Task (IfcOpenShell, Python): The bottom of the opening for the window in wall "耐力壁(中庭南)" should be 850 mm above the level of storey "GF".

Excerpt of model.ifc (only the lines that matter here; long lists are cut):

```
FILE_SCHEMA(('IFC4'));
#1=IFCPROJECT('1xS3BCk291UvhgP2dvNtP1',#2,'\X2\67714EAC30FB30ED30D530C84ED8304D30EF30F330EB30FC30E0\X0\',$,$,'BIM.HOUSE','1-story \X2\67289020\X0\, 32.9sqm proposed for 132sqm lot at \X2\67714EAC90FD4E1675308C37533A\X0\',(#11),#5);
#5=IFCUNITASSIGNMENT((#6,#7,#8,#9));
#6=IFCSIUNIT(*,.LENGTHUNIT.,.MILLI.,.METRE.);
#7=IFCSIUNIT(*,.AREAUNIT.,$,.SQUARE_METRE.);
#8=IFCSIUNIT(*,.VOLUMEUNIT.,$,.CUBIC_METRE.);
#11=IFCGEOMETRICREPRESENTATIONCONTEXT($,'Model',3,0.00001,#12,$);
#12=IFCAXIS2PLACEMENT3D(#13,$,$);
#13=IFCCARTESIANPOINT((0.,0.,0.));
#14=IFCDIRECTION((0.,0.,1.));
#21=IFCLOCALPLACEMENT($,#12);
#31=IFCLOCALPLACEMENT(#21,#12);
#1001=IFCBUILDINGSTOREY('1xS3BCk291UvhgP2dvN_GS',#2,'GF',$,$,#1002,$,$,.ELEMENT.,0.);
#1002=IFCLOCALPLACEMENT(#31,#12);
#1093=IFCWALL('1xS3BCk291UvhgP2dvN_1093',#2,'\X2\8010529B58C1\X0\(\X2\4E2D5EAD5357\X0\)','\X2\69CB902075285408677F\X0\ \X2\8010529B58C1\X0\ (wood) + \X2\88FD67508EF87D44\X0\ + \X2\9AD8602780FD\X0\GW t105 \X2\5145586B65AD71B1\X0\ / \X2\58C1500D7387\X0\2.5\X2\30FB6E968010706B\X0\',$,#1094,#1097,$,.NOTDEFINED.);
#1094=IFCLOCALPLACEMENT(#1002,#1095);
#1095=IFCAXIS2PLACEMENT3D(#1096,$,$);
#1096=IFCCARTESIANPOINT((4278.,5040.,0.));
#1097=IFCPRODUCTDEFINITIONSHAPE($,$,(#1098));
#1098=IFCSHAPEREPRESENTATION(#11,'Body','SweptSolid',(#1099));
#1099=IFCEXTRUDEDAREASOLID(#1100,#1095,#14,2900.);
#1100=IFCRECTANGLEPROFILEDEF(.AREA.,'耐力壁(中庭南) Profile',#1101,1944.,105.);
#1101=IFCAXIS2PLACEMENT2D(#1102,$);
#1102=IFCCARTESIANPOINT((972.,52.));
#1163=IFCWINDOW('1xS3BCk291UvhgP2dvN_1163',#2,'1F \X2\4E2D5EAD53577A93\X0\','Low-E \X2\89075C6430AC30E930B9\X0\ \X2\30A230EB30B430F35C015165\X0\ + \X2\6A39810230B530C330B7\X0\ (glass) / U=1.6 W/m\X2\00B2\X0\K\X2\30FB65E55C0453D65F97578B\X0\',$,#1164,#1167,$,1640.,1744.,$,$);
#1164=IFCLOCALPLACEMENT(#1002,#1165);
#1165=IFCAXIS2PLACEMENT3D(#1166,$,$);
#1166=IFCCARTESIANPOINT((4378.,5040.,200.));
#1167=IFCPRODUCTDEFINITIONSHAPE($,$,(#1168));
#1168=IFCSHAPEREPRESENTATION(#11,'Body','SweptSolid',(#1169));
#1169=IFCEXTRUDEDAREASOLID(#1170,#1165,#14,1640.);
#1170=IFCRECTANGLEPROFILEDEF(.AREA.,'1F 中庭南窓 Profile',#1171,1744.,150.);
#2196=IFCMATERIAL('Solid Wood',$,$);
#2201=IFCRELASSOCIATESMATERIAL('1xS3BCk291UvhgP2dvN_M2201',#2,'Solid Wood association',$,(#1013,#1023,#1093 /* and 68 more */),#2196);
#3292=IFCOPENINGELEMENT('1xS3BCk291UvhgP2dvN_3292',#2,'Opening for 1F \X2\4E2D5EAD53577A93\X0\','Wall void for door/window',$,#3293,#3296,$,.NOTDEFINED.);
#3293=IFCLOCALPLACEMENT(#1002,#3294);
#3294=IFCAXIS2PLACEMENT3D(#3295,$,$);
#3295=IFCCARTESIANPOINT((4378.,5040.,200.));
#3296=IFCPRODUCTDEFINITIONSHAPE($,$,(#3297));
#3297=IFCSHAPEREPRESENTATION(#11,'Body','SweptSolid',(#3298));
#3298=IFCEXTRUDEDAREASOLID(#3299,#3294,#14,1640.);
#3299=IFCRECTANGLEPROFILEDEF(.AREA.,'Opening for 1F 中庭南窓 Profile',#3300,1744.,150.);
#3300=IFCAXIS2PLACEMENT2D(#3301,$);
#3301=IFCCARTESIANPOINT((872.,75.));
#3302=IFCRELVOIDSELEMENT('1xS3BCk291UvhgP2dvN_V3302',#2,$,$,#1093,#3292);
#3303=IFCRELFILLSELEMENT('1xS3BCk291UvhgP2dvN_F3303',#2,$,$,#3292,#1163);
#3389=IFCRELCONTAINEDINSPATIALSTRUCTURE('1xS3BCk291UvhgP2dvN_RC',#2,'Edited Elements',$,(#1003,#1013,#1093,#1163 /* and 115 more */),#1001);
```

```python
import numpy as np
import ifcopenshell
import ifcopenshell.api.geometry
import ifcopenshell.geom
import ifcopenshell.util.element
import ifcopenshell.util.placement
import ifcopenshell.util.shape
import ifcopenshell.util.unit

model = ifcopenshell.open("model.ifc")
unit_scale = ifcopenshell.util.unit.calculate_unit_scale(model)

window = model.by_guid("1xS3BCk291UvhgP2dvN_1163")
opening = window.FillsVoids[0].RelatingOpeningElement
storey = ifcopenshell.util.element.get_container(window, ifc_class="IfcBuildingStorey")
level = ifcopenshell.util.placement.get_local_placement(storey.ObjectPlacement)[2, 3]

# The opening's origin need not be at the sill, so measure its lowest point.
shape = ifcopenshell.geom.create_shape(ifcopenshell.geom.settings(), opening)
bottom = ifcopenshell.util.shape.get_shape_bottom_elevation(shape, shape.geometry) / unit_scale
dz = level + 850.0 - bottom

shift = np.array([0.0, 0.0, dz])
# The window is not placed relative to its opening, so move both.
for product in (opening, window):
    matrix = ifcopenshell.util.placement.get_local_placement(product.ObjectPlacement)
    matrix[:3, 3] += shift
    ifcopenshell.api.geometry.edit_object_placement(model, product=product, matrix=matrix, is_si=False)

print(f"moved by {dz * unit_scale:+.3f} m")

model.write("model_updated.ifc")
```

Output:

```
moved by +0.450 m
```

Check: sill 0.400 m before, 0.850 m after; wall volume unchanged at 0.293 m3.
